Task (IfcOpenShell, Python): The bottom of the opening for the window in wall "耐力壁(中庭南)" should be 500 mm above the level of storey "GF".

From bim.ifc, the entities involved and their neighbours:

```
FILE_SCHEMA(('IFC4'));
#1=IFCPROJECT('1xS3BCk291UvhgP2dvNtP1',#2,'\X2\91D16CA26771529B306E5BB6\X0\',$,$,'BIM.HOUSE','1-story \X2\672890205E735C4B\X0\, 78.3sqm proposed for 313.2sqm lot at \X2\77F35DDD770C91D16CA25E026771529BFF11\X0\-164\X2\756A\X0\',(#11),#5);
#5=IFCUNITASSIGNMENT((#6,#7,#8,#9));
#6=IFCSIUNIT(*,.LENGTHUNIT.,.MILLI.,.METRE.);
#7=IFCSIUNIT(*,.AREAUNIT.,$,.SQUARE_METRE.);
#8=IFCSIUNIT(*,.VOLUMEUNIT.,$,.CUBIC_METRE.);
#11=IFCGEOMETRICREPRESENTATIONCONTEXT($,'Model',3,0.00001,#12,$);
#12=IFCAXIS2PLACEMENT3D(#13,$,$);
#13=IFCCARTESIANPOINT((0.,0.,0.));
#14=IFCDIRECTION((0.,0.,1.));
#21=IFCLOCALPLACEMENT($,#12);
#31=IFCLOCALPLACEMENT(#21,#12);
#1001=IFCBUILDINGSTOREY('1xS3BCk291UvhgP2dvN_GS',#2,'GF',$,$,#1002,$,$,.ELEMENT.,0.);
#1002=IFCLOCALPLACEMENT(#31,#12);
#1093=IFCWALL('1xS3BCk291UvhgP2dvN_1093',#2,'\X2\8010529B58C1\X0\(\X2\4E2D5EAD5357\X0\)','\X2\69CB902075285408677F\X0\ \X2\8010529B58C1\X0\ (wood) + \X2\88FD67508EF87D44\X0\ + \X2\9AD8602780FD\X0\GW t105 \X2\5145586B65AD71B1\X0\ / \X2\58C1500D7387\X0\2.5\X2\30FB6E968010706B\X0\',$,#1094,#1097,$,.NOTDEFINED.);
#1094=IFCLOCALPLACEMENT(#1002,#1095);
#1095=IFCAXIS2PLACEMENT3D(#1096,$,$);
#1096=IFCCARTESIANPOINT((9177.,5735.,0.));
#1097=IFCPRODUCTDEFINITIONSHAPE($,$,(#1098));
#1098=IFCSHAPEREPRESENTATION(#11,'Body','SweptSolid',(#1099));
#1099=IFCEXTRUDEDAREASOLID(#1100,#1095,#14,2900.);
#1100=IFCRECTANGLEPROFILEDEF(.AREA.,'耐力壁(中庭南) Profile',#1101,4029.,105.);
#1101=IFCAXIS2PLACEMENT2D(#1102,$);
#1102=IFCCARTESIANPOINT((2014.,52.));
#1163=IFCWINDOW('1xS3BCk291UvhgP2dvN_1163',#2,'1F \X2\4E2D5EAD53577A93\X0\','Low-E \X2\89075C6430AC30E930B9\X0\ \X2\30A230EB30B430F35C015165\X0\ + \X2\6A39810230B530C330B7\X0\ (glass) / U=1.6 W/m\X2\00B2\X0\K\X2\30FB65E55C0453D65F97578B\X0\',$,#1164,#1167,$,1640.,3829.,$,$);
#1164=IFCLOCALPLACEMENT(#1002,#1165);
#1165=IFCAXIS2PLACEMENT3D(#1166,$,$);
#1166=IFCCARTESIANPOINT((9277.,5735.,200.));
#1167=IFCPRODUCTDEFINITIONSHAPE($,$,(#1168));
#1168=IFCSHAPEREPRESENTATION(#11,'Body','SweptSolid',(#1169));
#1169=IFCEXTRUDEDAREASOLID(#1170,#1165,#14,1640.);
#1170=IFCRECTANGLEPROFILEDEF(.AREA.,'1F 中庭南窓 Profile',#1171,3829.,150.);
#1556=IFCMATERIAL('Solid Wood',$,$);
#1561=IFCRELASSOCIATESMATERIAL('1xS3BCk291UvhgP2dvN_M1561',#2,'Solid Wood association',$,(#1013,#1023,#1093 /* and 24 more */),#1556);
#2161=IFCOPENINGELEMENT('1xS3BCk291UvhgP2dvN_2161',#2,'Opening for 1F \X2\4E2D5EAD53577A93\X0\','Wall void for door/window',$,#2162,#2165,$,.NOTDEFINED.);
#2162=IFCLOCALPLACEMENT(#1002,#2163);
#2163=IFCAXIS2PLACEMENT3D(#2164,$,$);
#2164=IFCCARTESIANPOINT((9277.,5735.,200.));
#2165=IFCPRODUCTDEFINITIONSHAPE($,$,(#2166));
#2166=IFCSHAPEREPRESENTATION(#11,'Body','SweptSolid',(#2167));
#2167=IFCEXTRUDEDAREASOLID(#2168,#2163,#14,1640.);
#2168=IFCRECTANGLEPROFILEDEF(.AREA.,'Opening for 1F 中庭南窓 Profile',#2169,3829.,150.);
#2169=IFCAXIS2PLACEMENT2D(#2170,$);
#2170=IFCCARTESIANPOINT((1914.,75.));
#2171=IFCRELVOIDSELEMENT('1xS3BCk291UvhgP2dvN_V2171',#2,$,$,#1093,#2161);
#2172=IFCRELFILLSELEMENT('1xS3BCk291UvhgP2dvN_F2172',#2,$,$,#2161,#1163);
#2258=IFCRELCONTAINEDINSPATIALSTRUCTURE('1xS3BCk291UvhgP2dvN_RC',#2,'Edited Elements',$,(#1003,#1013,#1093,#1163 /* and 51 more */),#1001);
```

```python
import numpy as np
import ifcopenshell
import ifcopenshell.api.geometry
import ifcopenshell.geom
import ifcopenshell.util.element
import ifcopenshell.util.placement
import ifcopenshell.util.shape
import ifcopenshell.util.unit

model = ifcopenshell.open("bim.ifc")
unit_scale = ifcopenshell.util.unit.calculate_unit_scale(model)

window = model.by_guid("1xS3BCk291UvhgP2dvN_1163")
opening = window.FillsVoids[0].RelatingOpeningElement
storey = ifcopenshell.util.element.get_container(window, ifc_class="IfcBuildingStorey")
level = ifcopenshell.util.placement.get_local_placement(storey.ObjectPlacement)[2, 3]

# The opening's origin need not be at the sill, so measure its lowest point.
shape = ifcopenshell.geom.create_shape(ifcopenshell.geom.settings(), opening)
bottom = ifcopenshell.util.shape.get_shape_bottom_elevation(shape, shape.geometry) / unit_scale
dz = level + 500.0 - bottom

shift = np.array([0.0, 0.0, dz])
# The window is not placed relative to its opening, so move both.
for product in (opening, window):
    matrix = ifcopenshell.util.placement.get_local_placement(product.ObjectPlacement)
    matrix[:3, 3] += shift
    ifcopenshell.api.geometry.edit_object_placement(model, product=product, matrix=matrix, is_si=False)

print(f"moved by {dz * unit_scale:+.3f} m")

model.write("bim_v2.ifc")
```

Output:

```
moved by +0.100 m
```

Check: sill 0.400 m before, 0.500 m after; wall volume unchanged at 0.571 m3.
